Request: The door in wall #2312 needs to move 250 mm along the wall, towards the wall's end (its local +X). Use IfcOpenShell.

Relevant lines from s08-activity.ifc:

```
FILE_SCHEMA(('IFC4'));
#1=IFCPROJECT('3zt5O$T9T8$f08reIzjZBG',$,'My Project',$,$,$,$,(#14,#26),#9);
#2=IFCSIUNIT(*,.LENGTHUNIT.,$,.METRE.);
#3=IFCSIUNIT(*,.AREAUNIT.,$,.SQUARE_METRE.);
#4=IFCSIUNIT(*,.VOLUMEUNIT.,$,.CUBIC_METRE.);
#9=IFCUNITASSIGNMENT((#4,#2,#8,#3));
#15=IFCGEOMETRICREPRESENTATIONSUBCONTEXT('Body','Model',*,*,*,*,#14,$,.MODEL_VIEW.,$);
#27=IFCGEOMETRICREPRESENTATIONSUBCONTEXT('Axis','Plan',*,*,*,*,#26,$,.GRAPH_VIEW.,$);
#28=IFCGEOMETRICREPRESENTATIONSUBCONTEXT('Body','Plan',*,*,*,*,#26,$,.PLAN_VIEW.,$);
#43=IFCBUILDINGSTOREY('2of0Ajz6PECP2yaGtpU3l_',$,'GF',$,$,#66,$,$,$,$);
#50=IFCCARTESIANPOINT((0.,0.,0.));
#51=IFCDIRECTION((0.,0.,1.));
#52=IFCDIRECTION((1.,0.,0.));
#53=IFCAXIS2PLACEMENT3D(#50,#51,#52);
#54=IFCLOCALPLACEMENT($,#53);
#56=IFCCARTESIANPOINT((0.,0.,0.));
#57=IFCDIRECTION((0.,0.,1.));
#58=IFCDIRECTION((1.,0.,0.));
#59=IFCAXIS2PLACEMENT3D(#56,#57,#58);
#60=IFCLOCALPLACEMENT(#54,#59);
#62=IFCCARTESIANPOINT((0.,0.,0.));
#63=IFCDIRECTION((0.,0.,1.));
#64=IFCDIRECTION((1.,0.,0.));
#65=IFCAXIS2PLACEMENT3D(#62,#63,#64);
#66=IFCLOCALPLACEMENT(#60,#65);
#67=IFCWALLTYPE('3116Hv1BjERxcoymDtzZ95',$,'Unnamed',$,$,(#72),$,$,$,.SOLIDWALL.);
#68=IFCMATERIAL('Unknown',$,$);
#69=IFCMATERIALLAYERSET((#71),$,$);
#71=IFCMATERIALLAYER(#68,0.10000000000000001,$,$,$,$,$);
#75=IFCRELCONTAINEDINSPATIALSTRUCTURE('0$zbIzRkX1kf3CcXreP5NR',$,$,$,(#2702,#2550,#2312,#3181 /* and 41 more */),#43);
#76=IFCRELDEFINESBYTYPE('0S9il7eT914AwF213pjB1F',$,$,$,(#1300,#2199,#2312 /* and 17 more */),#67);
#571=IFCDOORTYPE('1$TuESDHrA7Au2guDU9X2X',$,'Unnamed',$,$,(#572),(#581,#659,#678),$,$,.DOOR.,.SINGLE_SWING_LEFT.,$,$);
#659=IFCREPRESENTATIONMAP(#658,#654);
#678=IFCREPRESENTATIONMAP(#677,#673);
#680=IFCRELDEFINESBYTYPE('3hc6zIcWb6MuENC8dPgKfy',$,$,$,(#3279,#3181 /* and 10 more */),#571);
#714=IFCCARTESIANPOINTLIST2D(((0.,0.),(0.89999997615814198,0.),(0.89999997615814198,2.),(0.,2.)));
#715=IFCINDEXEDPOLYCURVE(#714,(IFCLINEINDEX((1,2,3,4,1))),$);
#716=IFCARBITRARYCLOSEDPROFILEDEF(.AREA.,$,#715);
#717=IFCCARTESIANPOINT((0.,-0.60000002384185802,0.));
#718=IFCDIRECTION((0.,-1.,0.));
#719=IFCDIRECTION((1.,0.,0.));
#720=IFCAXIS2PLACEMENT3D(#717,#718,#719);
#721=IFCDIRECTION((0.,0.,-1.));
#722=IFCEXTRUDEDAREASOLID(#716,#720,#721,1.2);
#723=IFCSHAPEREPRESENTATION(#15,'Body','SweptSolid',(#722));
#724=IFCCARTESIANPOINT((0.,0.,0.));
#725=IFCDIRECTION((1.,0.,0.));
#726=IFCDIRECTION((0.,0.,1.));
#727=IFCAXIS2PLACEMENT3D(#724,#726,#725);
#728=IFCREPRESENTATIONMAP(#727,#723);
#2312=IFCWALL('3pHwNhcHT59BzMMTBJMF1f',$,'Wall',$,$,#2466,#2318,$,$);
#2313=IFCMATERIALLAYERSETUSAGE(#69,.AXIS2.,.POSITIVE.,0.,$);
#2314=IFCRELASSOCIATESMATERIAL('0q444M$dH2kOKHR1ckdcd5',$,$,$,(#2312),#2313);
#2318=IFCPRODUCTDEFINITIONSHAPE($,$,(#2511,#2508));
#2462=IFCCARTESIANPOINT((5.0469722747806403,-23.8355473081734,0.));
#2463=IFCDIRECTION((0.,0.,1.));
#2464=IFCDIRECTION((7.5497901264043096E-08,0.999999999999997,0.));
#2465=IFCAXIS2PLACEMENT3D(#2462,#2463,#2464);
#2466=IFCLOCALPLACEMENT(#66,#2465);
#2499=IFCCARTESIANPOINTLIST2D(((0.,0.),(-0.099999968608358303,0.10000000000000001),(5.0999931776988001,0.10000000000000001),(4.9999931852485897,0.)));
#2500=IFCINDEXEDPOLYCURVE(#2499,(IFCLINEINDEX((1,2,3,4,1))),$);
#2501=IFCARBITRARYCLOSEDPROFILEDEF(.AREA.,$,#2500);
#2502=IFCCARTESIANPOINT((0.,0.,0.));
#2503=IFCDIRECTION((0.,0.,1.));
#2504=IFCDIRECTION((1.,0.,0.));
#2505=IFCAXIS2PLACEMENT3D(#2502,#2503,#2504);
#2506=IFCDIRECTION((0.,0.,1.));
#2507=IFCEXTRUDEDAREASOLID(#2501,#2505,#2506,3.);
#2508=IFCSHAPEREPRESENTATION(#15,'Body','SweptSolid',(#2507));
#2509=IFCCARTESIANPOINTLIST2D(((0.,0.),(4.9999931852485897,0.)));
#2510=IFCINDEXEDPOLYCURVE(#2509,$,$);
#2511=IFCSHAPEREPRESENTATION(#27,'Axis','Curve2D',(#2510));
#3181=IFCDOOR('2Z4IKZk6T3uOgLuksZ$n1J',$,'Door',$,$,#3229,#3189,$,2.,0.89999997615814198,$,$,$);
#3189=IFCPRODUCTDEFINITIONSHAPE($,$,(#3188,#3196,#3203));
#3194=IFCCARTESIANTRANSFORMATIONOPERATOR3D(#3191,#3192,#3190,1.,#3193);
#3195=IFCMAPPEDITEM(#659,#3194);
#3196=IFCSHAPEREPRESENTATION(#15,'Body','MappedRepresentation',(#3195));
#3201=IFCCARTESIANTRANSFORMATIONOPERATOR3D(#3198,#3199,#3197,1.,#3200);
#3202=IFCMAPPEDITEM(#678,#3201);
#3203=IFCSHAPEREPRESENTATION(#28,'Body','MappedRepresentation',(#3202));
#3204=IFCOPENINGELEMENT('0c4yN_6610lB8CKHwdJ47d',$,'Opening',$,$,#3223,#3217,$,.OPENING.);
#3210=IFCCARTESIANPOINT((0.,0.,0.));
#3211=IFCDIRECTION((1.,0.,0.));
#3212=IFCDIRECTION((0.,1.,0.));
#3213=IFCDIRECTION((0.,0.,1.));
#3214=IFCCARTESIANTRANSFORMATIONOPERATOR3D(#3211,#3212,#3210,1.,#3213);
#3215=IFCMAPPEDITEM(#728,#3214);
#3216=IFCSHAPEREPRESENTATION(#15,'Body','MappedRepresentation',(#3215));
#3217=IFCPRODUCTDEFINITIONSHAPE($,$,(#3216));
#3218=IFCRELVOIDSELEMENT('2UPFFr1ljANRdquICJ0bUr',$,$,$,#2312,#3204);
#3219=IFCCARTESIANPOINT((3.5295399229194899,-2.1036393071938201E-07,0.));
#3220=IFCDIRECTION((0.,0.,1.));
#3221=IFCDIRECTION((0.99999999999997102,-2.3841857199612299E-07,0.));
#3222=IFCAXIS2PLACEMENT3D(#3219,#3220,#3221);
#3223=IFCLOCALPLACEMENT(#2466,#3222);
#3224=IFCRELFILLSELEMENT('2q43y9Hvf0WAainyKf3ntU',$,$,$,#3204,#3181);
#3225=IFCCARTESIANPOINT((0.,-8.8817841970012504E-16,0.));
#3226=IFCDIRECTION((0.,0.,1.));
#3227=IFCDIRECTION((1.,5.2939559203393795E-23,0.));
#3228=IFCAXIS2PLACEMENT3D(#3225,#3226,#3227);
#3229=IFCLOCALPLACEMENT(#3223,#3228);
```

```python
import ifcopenshell
import ifcopenshell.api.geometry
import ifcopenshell.util.placement
import ifcopenshell.util.unit

model = ifcopenshell.open("s08-activity.ifc")
unit_scale = ifcopenshell.util.unit.calculate_unit_scale(model)

door = model.by_id(3181)
opening = door.FillsVoids[0].RelatingOpeningElement
wall = opening.VoidsElements[0].RelatingBuildingElement

wall_matrix = ifcopenshell.util.placement.get_local_placement(wall.ObjectPlacement)
shift = wall_matrix[:3, 0] * 0.25 / unit_scale
before = ifcopenshell.util.placement.get_local_placement(door.ObjectPlacement)[:3, 3].copy()

# The door is placed relative to its opening, so it follows when the opening moves.
matrix = ifcopenshell.util.placement.get_local_placement(opening.ObjectPlacement)
matrix[:3, 3] += shift
ifcopenshell.api.geometry.edit_object_placement(
    model, product=opening, matrix=matrix, is_si=False, should_transform_children=True
)

after = ifcopenshell.util.placement.get_local_placement(door.ObjectPlacement)[:3, 3]
print("door moved by", (after - before).round(3) + 0.0)

model.write("s08-activity_v2.ifc")
```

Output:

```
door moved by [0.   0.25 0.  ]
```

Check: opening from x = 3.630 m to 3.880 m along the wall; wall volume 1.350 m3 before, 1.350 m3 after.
